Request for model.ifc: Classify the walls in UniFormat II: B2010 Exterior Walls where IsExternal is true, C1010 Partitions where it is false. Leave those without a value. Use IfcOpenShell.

First a look at what the model holds.

```python
import ifcopenshell
import ifcopenshell.util.element

model = ifcopenshell.open("model.ifc")
print(model.schema)
print("classifications:", [c.Name for c in model.by_type("IfcClassification")])
values = [ifcopenshell.util.element.get_pset(e, "Pset_WallCommon", "IsExternal") for e in model.by_type("IfcWall")]
for value in (True, False, None):
    print("IsExternal", value, values.count(value))
```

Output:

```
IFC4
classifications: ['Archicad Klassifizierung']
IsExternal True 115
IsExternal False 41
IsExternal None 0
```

```python
import ifcopenshell
import ifcopenshell.api.classification
import ifcopenshell.util.element

model = ifcopenshell.open("model.ifc")

system = ifcopenshell.api.classification.add_classification(model, classification="UniFormat II")

walls = model.by_type("IfcWall")
external = {e: ifcopenshell.util.element.get_pset(e, "Pset_WallCommon", "IsExternal") for e in walls}
for flag, code, name in ((True, "B2010", "Exterior Walls"), (False, "C1010", "Partitions")):
    products = [e for e in walls if external[e] is flag]
    ifcopenshell.api.classification.add_reference(
        model, products=products, classification=system, identification=code, name=name
    )
    print(code, len(products))

model.write("model_v2.ifc")
```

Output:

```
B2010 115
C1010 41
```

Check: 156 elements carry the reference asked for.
